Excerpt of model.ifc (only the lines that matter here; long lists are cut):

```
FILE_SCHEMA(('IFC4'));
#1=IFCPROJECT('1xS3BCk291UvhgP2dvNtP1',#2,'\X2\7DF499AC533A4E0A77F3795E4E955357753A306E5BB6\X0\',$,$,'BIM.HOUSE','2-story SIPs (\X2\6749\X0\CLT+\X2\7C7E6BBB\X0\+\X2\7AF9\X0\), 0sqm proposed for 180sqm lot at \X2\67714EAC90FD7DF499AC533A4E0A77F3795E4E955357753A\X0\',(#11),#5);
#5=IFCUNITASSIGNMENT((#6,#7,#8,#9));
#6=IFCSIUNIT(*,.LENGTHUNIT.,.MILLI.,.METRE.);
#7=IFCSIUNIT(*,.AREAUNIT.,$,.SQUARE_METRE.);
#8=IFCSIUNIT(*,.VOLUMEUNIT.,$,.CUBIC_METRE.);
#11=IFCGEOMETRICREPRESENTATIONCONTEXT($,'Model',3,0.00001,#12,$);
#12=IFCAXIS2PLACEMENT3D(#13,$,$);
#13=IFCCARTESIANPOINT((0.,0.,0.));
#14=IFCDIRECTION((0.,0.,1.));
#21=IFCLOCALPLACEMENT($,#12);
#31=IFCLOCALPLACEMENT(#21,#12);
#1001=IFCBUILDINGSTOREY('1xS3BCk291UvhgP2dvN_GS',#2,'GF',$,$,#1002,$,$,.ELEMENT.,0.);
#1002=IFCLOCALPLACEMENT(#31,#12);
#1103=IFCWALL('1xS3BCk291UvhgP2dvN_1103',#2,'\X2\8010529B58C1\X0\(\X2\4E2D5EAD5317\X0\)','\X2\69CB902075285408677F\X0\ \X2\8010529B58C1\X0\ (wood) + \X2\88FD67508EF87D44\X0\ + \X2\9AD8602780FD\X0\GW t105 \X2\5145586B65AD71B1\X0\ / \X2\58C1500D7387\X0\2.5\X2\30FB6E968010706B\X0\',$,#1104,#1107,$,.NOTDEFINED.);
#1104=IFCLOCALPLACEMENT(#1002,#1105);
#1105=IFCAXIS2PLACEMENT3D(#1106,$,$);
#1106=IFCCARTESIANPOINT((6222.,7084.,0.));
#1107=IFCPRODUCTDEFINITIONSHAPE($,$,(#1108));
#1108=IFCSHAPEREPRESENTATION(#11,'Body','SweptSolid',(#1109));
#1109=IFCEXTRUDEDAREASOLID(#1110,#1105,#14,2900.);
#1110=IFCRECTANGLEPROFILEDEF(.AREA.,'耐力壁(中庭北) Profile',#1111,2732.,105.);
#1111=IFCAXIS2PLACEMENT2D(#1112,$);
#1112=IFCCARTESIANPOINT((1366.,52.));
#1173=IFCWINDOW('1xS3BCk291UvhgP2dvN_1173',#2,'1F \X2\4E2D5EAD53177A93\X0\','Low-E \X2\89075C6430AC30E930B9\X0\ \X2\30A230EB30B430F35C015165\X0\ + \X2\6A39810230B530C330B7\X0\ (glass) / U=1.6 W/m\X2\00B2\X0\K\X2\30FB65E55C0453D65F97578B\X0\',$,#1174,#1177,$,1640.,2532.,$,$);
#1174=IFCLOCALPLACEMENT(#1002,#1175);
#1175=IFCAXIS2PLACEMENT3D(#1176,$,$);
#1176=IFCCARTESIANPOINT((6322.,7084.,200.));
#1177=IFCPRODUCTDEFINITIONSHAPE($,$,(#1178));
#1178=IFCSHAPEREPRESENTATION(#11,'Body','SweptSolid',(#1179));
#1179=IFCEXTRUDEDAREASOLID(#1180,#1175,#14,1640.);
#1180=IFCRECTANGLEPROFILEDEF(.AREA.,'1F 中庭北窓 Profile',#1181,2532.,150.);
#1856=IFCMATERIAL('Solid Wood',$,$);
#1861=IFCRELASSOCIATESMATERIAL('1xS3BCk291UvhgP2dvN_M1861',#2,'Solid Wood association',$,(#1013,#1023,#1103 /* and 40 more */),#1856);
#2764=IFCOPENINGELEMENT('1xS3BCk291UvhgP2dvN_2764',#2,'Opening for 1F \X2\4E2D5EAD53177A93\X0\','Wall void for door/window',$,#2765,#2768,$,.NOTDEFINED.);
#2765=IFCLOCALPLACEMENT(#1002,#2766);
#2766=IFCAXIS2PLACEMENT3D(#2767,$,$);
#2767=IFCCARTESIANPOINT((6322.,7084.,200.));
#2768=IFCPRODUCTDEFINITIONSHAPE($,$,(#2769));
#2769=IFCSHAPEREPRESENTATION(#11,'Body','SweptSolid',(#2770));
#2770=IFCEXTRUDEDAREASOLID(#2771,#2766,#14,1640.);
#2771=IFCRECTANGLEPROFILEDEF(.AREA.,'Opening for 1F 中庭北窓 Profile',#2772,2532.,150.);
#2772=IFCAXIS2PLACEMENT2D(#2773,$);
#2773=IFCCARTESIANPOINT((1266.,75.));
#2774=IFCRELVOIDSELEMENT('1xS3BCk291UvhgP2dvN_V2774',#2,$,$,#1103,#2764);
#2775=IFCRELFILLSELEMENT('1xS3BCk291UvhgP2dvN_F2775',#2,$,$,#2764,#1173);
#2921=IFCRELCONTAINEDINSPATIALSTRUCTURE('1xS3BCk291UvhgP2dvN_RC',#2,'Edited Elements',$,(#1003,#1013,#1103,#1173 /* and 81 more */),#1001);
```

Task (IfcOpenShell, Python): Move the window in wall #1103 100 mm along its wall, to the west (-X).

```python
import ifcopenshell
import ifcopenshell.api.geometry
import ifcopenshell.util.placement
import ifcopenshell.util.unit

model = ifcopenshell.open("model.ifc")
unit_scale = ifcopenshell.util.unit.calculate_unit_scale(model)

window = model.by_guid("1xS3BCk291UvhgP2dvN_1173")
opening = window.FillsVoids[0].RelatingOpeningElement
wall = opening.VoidsElements[0].RelatingBuildingElement

wall_matrix = ifcopenshell.util.placement.get_local_placement(wall.ObjectPlacement)
shift = wall_matrix[:3, 0] * -0.1 / unit_scale
before = ifcopenshell.util.placement.get_local_placement(window.ObjectPlacement)[:3, 3].copy()

# The window is not placed relative to its opening, so move both.
for product in (opening, window):
    matrix = ifcopenshell.util.placement.get_local_placement(product.ObjectPlacement)
    matrix[:3, 3] += shift
    ifcopenshell.api.geometry.edit_object_placement(model, product=product, matrix=matrix, is_si=False)

after = ifcopenshell.util.placement.get_local_placement(window.ObjectPlacement)[:3, 3]
print("window moved by", (after - before).round(3) + 0.0)

model.write("model_edited.ifc")
```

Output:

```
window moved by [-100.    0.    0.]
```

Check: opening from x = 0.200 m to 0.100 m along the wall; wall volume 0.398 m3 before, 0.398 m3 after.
